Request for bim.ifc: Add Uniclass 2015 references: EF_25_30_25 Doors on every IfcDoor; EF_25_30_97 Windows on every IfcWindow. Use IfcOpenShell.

First a look at what the model holds.

```python
import ifcopenshell

model = ifcopenshell.open("bim.ifc")
print(model.schema)
print("classifications:", [c.Name for c in model.by_type("IfcClassification")])
for ifc_class in ("IfcDoor", "IfcRoof", "IfcStair", "IfcWall", "IfcWindow"):
    print(ifc_class, len(model.by_type(ifc_class)))
```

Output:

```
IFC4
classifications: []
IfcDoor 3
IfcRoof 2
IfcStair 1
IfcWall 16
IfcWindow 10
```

```python
import ifcopenshell
import ifcopenshell.api.classification

model = ifcopenshell.open("bim.ifc")

system = ifcopenshell.api.classification.add_classification(model, classification="Uniclass 2015")

codes = {
    "IfcDoor": ("EF_25_30_25", "Doors"),
    "IfcWindow": ("EF_25_30_97", "Windows"),
}
for ifc_class, (code, name) in codes.items():
    products = model.by_type(ifc_class)
    ifcopenshell.api.classification.add_reference(
        model, products=products, classification=system, identification=code, name=name
    )
    print(code, len(products))

model.write("bim_edited.ifc")
```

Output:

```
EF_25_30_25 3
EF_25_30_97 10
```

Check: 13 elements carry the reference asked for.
